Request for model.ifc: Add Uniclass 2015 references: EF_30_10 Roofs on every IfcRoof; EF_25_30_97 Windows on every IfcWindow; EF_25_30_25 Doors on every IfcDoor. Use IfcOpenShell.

First a look at what the model holds.

```python
import ifcopenshell

model = ifcopenshell.open("model.ifc")
print(model.schema)
print("classifications:", [c.Name for c in model.by_type("IfcClassification")])
for ifc_class in ("IfcDoor", "IfcRoof", "IfcStair", "IfcWall", "IfcWindow"):
    print(ifc_class, len(model.by_type(ifc_class)))
```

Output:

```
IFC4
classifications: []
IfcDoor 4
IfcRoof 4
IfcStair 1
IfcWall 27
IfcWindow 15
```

```python
import ifcopenshell
import ifcopenshell.api.classification

model = ifcopenshell.open("model.ifc")

system = ifcopenshell.api.classification.add_classification(model, classification="Uniclass 2015")

codes = {
    "IfcRoof": ("EF_30_10", "Roofs"),
    "IfcWindow": ("EF_25_30_97", "Windows"),
    "IfcDoor": ("EF_25_30_25", "Doors"),
}
for ifc_class, (code, name) in codes.items():
    products = model.by_type(ifc_class)
    ifcopenshell.api.classification.add_reference(
        model, products=products, classification=system, identification=code, name=name
    )
    print(code, len(products))

model.write("model_updated.ifc")
```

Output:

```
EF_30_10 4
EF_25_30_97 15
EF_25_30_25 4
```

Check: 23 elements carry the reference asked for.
